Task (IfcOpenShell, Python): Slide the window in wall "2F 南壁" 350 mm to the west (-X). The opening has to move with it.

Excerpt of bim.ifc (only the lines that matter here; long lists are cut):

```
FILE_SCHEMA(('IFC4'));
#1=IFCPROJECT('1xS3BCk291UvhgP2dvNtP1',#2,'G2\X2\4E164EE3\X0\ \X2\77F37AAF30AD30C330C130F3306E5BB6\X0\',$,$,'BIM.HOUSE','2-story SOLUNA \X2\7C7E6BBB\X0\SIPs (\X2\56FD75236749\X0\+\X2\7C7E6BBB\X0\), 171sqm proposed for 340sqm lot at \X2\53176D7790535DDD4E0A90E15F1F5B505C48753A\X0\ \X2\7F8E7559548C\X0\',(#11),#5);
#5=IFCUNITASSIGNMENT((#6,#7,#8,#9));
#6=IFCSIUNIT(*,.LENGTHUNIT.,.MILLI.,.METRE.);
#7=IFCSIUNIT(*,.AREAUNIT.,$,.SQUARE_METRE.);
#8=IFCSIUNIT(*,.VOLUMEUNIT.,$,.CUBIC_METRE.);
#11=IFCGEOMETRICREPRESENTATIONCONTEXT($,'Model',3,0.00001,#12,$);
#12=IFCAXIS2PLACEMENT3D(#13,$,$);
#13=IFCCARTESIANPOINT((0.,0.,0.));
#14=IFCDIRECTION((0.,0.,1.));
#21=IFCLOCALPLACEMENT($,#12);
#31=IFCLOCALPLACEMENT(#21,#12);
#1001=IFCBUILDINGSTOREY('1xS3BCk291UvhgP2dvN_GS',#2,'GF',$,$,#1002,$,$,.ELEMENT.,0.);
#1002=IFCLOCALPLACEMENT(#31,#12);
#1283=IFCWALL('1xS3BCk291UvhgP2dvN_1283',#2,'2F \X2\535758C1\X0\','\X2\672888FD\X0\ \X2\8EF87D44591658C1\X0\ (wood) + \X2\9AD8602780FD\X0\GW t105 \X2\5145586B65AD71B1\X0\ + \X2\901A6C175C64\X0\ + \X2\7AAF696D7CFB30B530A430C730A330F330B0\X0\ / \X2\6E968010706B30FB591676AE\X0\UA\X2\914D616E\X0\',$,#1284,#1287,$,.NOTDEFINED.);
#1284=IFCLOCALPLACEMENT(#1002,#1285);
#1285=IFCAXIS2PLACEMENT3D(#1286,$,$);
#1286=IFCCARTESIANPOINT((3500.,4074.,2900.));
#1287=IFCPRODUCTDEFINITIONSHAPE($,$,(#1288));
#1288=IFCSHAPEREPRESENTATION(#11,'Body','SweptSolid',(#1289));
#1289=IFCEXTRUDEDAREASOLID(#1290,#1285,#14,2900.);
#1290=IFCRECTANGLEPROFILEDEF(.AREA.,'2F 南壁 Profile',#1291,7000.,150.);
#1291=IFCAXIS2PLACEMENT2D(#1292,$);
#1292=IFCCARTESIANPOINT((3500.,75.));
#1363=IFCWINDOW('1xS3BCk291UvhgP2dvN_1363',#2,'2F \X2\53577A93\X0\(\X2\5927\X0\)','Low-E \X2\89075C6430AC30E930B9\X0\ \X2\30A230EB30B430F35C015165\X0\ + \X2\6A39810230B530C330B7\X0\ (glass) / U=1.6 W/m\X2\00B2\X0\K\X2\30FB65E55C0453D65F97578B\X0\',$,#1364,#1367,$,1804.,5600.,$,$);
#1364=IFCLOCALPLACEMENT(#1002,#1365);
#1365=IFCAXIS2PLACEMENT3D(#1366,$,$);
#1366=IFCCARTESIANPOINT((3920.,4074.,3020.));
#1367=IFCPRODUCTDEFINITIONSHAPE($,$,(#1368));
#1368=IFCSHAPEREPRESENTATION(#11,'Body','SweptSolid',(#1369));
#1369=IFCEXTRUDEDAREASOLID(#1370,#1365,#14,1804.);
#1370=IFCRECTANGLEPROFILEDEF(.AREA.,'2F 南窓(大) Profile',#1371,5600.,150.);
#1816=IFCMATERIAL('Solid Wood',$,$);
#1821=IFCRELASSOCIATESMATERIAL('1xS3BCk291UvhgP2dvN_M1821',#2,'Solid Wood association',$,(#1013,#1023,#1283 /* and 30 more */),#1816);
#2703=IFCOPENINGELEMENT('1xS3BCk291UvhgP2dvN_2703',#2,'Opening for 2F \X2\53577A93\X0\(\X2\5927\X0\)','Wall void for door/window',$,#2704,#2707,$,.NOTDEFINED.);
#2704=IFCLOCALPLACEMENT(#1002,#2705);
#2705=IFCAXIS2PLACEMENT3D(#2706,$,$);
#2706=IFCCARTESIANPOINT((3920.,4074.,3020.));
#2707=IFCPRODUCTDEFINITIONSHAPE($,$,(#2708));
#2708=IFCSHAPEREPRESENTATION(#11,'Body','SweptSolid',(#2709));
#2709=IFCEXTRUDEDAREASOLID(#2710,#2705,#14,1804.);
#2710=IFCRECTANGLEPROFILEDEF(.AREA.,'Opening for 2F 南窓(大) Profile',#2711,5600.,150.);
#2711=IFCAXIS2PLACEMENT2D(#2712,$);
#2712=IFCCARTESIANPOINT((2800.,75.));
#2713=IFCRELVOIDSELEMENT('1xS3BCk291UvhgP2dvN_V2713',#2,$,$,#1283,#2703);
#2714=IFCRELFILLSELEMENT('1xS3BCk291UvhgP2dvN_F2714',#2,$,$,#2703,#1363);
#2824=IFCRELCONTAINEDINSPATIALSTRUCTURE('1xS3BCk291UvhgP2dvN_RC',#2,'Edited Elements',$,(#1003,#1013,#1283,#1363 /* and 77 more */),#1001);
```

```python
import ifcopenshell
import ifcopenshell.api.geometry
import ifcopenshell.util.placement
import ifcopenshell.util.unit

model = ifcopenshell.open("bim.ifc")
unit_scale = ifcopenshell.util.unit.calculate_unit_scale(model)

window = model.by_guid("1xS3BCk291UvhgP2dvN_1363")
opening = window.FillsVoids[0].RelatingOpeningElement
wall = opening.VoidsElements[0].RelatingBuildingElement

wall_matrix = ifcopenshell.util.placement.get_local_placement(wall.ObjectPlacement)
shift = wall_matrix[:3, 0] * -0.35 / unit_scale
before = ifcopenshell.util.placement.get_local_placement(window.ObjectPlacement)[:3, 3].copy()

# The window is not placed relative to its opening, so move both.
for product in (opening, window):
    matrix = ifcopenshell.util.placement.get_local_placement(product.ObjectPlacement)
    matrix[:3, 3] += shift
    ifcopenshell.api.geometry.edit_object_placement(model, product=product, matrix=matrix, is_si=False)

after = ifcopenshell.util.placement.get_local_placement(window.ObjectPlacement)[:3, 3]
print("window moved by", (after - before).round(3) + 0.0)

model.write("bim_rev.ifc")
```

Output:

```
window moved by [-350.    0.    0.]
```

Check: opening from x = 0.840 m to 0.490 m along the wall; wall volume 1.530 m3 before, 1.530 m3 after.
